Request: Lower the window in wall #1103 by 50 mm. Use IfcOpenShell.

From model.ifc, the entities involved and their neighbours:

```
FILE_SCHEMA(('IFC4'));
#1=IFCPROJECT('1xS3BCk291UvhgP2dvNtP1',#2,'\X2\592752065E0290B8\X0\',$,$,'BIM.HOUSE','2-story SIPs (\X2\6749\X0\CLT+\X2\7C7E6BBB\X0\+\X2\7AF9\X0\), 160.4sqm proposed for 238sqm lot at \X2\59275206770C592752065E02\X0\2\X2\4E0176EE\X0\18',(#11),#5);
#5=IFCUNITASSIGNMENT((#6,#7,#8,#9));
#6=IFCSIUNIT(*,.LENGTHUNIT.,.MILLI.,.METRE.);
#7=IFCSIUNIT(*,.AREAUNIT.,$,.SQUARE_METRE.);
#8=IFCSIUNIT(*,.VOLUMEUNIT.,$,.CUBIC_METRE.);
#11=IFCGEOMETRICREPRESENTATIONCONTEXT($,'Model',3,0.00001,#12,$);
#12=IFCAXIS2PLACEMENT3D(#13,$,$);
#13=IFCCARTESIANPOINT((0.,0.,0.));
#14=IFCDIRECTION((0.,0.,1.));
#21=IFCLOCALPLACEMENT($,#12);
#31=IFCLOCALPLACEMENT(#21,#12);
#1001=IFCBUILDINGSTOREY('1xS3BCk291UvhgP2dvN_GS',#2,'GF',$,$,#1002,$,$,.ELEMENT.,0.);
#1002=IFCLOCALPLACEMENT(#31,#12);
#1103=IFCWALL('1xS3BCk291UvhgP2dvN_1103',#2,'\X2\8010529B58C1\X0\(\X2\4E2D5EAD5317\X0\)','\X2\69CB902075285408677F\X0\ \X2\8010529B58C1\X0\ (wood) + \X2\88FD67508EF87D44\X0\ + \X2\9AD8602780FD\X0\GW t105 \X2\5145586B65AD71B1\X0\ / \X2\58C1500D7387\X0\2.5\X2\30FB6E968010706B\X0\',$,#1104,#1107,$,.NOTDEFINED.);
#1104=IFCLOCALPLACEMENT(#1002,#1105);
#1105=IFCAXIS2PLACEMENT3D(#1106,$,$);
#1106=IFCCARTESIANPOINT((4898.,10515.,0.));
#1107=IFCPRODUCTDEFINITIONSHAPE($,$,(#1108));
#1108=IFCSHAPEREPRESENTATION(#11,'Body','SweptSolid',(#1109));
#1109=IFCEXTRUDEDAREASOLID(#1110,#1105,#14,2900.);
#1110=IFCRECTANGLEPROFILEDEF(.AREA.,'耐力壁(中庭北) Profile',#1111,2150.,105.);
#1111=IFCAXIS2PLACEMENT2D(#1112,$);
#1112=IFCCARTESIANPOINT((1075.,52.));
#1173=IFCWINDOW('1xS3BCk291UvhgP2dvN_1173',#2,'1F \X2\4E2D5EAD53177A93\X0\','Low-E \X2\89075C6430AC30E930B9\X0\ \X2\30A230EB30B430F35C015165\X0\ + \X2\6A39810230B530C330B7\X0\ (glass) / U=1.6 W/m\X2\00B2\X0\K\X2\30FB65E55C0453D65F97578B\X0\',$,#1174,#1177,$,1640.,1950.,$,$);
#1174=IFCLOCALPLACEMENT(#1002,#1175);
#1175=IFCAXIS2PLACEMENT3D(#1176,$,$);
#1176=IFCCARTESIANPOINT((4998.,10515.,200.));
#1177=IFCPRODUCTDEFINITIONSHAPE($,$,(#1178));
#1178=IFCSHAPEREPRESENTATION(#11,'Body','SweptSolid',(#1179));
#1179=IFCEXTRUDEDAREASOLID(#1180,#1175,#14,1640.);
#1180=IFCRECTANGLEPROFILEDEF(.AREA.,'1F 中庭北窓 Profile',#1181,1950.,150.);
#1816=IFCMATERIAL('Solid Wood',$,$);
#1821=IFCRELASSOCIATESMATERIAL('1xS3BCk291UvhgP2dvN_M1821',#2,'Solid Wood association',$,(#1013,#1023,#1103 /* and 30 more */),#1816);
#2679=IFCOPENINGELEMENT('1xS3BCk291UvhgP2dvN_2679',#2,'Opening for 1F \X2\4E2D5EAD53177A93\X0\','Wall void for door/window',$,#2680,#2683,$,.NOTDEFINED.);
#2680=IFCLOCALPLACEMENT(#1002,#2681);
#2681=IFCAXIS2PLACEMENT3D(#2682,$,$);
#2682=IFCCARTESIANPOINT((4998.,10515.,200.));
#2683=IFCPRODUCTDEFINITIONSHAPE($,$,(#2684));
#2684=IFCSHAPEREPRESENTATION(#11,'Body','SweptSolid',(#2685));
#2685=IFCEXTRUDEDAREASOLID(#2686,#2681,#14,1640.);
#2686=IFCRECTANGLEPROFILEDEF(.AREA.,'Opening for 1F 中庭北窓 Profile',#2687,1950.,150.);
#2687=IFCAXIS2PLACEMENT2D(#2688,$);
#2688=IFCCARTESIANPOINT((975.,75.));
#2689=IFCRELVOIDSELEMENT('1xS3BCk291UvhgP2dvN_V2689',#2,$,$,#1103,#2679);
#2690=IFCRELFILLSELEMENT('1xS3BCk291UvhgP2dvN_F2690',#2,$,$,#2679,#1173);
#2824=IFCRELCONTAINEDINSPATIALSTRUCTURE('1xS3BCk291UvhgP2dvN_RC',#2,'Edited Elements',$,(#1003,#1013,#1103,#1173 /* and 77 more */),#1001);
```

```python
import numpy as np
import ifcopenshell
import ifcopenshell.api.geometry
import ifcopenshell.util.placement
import ifcopenshell.util.unit

model = ifcopenshell.open("model.ifc")
unit_scale = ifcopenshell.util.unit.calculate_unit_scale(model)

window = model.by_guid("1xS3BCk291UvhgP2dvN_1173")
opening = window.FillsVoids[0].RelatingOpeningElement
dz = -0.05 / unit_scale

shift = np.array([0.0, 0.0, dz])
# The window is not placed relative to its opening, so move both.
for product in (opening, window):
    matrix = ifcopenshell.util.placement.get_local_placement(product.ObjectPlacement)
    matrix[:3, 3] += shift
    ifcopenshell.api.geometry.edit_object_placement(model, product=product, matrix=matrix, is_si=False)

print(f"moved by {dz * unit_scale:+.3f} m")

model.write("model_updated.ifc")
```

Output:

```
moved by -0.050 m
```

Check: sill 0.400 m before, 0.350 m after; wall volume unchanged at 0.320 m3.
